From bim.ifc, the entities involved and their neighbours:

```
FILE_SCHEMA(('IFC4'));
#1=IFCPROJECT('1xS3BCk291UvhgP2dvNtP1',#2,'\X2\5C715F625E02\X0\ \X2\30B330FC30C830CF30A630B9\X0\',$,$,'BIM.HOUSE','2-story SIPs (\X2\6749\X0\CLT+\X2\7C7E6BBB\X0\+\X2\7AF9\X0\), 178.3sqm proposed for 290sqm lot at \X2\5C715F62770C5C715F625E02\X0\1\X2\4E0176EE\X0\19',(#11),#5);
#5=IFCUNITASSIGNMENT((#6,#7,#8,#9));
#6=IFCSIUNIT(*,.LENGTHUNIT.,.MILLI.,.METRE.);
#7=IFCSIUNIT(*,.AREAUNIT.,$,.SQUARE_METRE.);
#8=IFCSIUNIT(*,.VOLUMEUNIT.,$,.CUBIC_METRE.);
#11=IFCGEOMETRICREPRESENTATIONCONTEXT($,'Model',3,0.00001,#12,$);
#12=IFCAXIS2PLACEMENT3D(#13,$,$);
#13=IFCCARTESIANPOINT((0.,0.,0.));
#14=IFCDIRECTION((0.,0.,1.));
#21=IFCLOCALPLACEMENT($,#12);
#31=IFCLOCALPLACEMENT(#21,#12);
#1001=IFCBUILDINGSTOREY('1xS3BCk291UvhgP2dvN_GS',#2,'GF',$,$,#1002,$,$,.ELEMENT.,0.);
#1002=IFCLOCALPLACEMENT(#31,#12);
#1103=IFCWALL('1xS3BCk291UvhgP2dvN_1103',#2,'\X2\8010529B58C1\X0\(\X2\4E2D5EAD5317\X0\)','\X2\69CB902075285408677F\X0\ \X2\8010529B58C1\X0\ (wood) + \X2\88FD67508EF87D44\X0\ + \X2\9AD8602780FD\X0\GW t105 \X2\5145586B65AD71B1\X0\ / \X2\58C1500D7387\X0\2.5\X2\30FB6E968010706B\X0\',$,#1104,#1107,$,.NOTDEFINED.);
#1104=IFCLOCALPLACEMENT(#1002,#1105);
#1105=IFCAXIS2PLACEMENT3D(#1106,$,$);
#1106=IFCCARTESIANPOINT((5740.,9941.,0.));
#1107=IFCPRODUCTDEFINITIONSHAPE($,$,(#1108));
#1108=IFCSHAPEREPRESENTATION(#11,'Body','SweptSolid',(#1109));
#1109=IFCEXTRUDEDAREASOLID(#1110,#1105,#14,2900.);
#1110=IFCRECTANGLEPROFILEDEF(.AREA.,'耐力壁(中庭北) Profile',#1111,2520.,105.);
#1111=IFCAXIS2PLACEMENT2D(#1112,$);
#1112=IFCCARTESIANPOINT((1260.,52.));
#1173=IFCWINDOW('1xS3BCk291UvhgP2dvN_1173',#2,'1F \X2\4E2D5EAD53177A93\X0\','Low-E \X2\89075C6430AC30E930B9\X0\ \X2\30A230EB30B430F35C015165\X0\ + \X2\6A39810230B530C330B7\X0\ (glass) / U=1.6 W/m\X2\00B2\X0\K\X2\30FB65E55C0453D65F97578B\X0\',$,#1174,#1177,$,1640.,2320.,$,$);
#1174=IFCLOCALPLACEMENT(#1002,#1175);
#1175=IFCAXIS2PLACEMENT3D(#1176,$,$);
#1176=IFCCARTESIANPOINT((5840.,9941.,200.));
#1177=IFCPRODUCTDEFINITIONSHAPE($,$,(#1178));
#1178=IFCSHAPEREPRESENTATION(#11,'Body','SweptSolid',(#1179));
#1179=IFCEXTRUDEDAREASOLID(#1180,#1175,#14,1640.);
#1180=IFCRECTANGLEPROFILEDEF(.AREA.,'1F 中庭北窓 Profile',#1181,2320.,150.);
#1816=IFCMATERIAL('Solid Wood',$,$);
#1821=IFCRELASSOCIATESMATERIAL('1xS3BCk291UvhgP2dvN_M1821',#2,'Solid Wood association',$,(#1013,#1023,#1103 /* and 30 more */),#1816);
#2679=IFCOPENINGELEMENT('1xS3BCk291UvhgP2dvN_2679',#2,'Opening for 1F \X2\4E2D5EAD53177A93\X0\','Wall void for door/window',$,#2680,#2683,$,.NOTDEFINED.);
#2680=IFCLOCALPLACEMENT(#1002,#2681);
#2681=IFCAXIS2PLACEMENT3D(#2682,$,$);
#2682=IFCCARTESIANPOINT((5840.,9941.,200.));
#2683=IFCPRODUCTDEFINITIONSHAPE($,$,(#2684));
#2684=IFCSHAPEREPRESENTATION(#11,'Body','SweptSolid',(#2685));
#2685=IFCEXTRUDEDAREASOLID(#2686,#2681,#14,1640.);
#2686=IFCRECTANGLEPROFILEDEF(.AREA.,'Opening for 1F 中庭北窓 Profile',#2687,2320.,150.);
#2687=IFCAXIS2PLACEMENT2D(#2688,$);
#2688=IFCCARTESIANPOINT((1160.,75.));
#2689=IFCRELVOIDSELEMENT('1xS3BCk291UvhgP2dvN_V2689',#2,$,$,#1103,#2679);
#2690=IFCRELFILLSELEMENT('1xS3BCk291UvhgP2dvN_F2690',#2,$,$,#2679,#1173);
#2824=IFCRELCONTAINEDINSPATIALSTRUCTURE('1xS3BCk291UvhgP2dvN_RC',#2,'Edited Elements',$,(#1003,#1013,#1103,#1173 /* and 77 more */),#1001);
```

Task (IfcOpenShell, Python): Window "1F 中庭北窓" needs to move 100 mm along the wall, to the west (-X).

```python
import ifcopenshell
import ifcopenshell.api.geometry
import ifcopenshell.util.placement

model = ifcopenshell.open("bim.ifc")

window = model.by_guid("1xS3BCk291UvhgP2dvN_1173")
opening = window.FillsVoids[0].RelatingOpeningElement
wall = opening.VoidsElements[0].RelatingBuildingElement

wall_matrix = ifcopenshell.util.placement.get_local_placement(wall.ObjectPlacement)
shift = wall_matrix[:3, 0] * -100.0
before = ifcopenshell.util.placement.get_local_placement(window.ObjectPlacement)[:3, 3].copy()

# The window is not placed relative to its opening, so move both.
for product in (opening, window):
    matrix = ifcopenshell.util.placement.get_local_placement(product.ObjectPlacement)
    matrix[:3, 3] += shift
    ifcopenshell.api.geometry.edit_object_placement(model, product=product, matrix=matrix, is_si=False)

after = ifcopenshell.util.placement.get_local_placement(window.ObjectPlacement)[:3, 3]
print("window moved by", (after - before).round(3) + 0.0)

model.write("bim_updated.ifc")
```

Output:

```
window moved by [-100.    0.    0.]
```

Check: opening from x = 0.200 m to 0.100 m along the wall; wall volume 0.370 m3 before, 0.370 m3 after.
